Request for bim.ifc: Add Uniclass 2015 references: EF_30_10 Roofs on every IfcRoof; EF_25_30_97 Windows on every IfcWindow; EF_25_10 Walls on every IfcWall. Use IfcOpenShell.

First a look at what the model holds.

```python
import ifcopenshell

model = ifcopenshell.open("bim.ifc")
print(model.schema)
print("classifications:", [c.Name for c in model.by_type("IfcClassification")])
for ifc_class in ("IfcDoor", "IfcRoof", "IfcStair", "IfcWall", "IfcWindow"):
    print(ifc_class, len(model.by_type(ifc_class)))
```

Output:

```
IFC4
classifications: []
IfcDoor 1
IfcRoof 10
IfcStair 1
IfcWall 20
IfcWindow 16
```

```python
import ifcopenshell
import ifcopenshell.api.classification

model = ifcopenshell.open("bim.ifc")

system = ifcopenshell.api.classification.add_classification(model, classification="Uniclass 2015")

codes = {
    "IfcRoof": ("EF_30_10", "Roofs"),
    "IfcWindow": ("EF_25_30_97", "Windows"),
    "IfcWall": ("EF_25_10", "Walls"),
}
for ifc_class, (code, name) in codes.items():
    products = model.by_type(ifc_class)
    ifcopenshell.api.classification.add_reference(
        model, products=products, classification=system, identification=code, name=name
    )
    print(code, len(products))

model.write("bim_rev.ifc")
```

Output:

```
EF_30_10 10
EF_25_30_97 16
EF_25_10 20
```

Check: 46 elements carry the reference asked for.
